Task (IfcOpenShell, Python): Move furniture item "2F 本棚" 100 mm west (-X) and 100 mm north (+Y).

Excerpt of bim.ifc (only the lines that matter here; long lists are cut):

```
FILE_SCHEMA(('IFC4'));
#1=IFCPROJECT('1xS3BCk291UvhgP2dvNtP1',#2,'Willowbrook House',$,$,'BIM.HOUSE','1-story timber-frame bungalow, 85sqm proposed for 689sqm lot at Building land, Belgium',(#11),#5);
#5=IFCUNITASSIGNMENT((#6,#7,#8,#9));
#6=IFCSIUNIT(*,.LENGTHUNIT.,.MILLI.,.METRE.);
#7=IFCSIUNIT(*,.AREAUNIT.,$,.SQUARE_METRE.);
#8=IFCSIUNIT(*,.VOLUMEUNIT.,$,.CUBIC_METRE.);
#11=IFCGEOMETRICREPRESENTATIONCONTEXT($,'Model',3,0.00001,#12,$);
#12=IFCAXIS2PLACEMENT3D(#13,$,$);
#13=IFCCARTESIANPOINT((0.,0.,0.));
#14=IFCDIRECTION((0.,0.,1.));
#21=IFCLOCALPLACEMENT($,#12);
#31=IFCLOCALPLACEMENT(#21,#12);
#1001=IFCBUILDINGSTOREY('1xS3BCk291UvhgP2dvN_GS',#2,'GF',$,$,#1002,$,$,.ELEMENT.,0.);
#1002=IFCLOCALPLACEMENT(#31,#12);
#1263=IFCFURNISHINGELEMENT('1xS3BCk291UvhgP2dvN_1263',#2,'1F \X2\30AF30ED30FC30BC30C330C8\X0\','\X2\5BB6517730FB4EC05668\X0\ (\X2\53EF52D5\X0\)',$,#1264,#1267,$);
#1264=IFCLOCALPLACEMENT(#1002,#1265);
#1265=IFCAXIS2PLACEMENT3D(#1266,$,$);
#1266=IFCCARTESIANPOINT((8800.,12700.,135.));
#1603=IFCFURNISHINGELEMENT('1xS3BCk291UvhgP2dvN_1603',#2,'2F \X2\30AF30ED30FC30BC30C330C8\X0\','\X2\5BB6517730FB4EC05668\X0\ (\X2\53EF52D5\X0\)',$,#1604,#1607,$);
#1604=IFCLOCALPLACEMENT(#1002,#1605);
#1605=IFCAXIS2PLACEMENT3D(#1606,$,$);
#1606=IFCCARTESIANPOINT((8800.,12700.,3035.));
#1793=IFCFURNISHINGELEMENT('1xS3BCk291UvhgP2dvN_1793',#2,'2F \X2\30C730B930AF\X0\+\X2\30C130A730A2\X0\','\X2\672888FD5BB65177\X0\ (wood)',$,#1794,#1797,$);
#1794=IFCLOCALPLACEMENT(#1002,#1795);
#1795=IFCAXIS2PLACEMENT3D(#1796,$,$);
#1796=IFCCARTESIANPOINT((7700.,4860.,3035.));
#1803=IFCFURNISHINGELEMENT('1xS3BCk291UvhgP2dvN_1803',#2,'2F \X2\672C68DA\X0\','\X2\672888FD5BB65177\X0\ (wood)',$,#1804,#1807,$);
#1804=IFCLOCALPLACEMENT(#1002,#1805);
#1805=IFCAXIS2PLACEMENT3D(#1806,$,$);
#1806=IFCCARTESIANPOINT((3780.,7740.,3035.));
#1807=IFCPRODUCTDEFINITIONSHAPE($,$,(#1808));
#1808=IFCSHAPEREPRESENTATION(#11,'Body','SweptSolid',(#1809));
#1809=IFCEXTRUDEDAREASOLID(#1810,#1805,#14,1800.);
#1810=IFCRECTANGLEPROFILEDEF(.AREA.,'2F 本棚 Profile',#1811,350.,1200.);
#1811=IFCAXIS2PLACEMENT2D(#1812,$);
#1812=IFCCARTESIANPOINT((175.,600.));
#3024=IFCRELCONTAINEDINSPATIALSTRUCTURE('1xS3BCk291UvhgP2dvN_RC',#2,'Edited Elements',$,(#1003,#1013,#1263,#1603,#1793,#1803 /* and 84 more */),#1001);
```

```python
import ifcopenshell
import ifcopenshell.api.geometry
import ifcopenshell.util.placement
import ifcopenshell.util.unit

model = ifcopenshell.open("bim.ifc")
unit_scale = ifcopenshell.util.unit.calculate_unit_scale(model)

item = model.by_guid("1xS3BCk291UvhgP2dvN_1803")
matrix = ifcopenshell.util.placement.get_local_placement(item.ObjectPlacement)
matrix[0, 3] -= 0.1 / unit_scale
matrix[1, 3] += 0.1 / unit_scale
ifcopenshell.api.geometry.edit_object_placement(model, product=item, matrix=matrix, is_si=False)

print(ifcopenshell.util.placement.get_local_placement(item.ObjectPlacement).round(3) + 0.0)

model.write("bim_updated.ifc")
```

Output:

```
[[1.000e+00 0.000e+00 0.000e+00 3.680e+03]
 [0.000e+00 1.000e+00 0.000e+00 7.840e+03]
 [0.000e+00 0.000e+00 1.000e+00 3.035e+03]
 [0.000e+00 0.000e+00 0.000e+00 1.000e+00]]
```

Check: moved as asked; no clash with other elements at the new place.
